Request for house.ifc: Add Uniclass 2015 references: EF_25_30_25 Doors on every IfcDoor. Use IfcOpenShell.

First a look at what the model holds.

```python
import ifcopenshell

model = ifcopenshell.open("house.ifc")
print(model.schema)
print("classifications:", [c.Name for c in model.by_type("IfcClassification")])
for ifc_class in ("IfcDoor", "IfcRoof", "IfcStair", "IfcWall", "IfcWindow"):
    print(ifc_class, len(model.by_type(ifc_class)))
```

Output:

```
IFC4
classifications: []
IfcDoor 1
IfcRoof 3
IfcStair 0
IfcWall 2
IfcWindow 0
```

```python
import ifcopenshell
import ifcopenshell.api.classification

model = ifcopenshell.open("house.ifc")

system = ifcopenshell.api.classification.add_classification(model, classification="Uniclass 2015")

codes = {
    "IfcDoor": ("EF_25_30_25", "Doors"),
}
for ifc_class, (code, name) in codes.items():
    products = model.by_type(ifc_class)
    ifcopenshell.api.classification.add_reference(
        model, products=products, classification=system, identification=code, name=name
    )
    print(code, len(products))

model.write("house_v2.ifc")
```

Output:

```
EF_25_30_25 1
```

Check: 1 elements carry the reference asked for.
